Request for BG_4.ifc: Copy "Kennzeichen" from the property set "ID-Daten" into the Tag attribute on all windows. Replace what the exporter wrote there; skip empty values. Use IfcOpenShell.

First a look at what the model holds.

```python
import ifcopenshell
import ifcopenshell.util.element

model = ifcopenshell.open("BG_4.ifc")
print(model.schema)
windows = model.by_type("IfcWindow")
print(len(windows), "windows")
for e in windows[:8]:
    source = ifcopenshell.util.element.get_pset(e, "ID-Daten", "Kennzeichen")
    target = e.Tag
    print(e.id(), repr(source), repr(target), sep=" | ")
```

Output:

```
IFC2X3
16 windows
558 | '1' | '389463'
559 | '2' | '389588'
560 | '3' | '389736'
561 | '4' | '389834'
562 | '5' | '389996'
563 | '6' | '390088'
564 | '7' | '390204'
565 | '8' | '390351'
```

```python
import ifcopenshell
import ifcopenshell.util.element

model = ifcopenshell.open("BG_4.ifc")

count = 0
for e in model.by_type("IfcWindow"):
    value = ifcopenshell.util.element.get_pset(e, "ID-Daten", "Kennzeichen")
    current = e.Tag
    if not value or not value.strip() or current == value:
        continue
    e.Tag = value
    count += 1

print(count, "windows updated")

model.write("BG_4_edited.ifc")
```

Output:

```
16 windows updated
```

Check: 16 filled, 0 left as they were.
